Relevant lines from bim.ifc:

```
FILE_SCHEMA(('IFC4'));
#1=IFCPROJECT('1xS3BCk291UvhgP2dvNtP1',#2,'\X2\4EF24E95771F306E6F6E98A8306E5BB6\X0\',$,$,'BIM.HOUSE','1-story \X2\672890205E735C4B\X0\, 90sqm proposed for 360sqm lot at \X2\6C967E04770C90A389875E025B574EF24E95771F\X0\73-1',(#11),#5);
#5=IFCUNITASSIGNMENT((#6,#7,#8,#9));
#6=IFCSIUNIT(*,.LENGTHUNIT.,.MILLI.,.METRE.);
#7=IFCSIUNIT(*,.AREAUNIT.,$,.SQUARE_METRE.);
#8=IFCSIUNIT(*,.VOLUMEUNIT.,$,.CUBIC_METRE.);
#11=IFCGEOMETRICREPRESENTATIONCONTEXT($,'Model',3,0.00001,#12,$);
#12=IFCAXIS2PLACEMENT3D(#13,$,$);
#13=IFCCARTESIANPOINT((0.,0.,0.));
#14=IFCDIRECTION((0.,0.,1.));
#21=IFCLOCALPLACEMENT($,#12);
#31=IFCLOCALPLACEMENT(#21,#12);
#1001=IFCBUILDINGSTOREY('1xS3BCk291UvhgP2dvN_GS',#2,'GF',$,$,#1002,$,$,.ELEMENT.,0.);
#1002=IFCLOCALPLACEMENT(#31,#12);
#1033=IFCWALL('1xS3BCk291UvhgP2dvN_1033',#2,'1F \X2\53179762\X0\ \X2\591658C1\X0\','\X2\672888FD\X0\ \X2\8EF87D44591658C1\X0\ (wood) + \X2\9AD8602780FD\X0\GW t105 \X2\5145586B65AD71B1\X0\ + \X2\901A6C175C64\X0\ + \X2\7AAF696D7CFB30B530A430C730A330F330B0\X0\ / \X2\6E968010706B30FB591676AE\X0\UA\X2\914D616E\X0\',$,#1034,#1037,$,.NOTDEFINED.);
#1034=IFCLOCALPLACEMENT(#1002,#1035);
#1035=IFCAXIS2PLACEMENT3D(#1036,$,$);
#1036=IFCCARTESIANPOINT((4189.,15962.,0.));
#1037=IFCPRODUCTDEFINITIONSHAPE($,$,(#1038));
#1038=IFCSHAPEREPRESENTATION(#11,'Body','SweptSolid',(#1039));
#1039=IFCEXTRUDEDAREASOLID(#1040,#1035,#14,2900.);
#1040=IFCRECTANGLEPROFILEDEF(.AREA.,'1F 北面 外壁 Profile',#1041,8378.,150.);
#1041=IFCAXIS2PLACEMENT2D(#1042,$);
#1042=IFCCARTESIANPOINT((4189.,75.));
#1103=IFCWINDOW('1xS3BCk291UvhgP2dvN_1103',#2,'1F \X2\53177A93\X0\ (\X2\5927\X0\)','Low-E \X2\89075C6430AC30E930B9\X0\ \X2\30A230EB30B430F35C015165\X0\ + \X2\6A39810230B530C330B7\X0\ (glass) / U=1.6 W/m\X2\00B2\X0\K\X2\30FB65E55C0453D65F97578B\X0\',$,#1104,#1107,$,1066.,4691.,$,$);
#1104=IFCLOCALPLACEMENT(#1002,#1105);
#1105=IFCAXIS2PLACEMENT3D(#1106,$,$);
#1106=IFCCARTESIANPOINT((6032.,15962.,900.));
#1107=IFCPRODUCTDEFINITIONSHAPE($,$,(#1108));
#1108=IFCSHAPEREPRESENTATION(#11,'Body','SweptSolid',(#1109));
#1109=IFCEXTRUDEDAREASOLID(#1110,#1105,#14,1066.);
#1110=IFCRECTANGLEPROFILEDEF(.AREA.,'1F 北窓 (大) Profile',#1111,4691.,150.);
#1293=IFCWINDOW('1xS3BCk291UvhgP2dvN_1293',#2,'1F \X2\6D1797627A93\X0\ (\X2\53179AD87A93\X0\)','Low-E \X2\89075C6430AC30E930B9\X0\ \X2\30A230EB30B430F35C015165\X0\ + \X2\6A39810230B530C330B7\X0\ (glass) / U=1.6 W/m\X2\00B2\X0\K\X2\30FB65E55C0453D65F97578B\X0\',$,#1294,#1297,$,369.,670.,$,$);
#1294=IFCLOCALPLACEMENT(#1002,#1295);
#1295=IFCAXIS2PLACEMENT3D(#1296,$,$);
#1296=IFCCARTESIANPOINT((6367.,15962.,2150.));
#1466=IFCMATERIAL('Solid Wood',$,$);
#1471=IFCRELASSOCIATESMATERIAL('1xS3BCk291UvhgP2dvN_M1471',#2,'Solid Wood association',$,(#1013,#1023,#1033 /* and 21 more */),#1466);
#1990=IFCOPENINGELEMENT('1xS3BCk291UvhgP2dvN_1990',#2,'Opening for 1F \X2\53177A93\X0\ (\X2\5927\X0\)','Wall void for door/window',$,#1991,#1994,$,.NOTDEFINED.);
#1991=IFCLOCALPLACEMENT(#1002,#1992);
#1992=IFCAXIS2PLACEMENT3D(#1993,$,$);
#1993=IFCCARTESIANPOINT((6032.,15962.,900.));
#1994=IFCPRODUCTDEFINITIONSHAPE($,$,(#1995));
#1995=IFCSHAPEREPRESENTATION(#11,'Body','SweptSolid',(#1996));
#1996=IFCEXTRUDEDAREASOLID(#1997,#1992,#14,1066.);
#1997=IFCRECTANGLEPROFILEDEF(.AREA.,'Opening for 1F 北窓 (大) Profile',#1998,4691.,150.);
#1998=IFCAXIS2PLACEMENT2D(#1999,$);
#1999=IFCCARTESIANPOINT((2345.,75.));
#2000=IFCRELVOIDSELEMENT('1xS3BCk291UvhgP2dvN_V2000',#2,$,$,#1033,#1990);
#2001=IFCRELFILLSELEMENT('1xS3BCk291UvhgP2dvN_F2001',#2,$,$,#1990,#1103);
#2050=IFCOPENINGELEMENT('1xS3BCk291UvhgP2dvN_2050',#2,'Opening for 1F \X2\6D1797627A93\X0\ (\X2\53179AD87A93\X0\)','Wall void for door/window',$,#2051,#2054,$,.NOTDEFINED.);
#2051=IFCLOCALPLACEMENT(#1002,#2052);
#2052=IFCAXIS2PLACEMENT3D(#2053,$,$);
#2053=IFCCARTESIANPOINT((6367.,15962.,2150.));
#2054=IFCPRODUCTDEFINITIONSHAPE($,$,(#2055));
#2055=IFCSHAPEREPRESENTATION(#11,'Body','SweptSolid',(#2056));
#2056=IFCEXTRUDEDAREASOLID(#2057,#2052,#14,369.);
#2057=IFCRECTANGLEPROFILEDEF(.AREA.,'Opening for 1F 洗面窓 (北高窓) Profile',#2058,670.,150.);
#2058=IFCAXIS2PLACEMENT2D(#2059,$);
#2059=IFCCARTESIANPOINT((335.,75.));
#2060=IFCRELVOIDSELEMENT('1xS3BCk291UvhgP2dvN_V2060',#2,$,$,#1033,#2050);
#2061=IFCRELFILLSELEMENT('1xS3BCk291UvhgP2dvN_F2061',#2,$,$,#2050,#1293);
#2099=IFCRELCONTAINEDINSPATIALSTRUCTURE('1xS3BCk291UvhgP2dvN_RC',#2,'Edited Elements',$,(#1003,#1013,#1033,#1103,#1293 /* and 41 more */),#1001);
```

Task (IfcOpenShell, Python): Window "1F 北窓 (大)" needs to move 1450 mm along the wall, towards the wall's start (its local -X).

```python
import ifcopenshell
import ifcopenshell.api.geometry
import ifcopenshell.util.placement
import ifcopenshell.util.unit

model = ifcopenshell.open("bim.ifc")
unit_scale = ifcopenshell.util.unit.calculate_unit_scale(model)

window = model.by_guid("1xS3BCk291UvhgP2dvN_1103")
opening = window.FillsVoids[0].RelatingOpeningElement
wall = opening.VoidsElements[0].RelatingBuildingElement

wall_matrix = ifcopenshell.util.placement.get_local_placement(wall.ObjectPlacement)
shift = wall_matrix[:3, 0] * -1.45 / unit_scale
before = ifcopenshell.util.placement.get_local_placement(window.ObjectPlacement)[:3, 3].copy()

# The window is not placed relative to its opening, so move both.
for product in (opening, window):
    matrix = ifcopenshell.util.placement.get_local_placement(product.ObjectPlacement)
    matrix[:3, 3] += shift
    ifcopenshell.api.geometry.edit_object_placement(model, product=product, matrix=matrix, is_si=False)

after = ifcopenshell.util.placement.get_local_placement(window.ObjectPlacement)[:3, 3]
print("window moved by", (after - before).round(3) + 0.0)

model.write("bim_updated.ifc")
```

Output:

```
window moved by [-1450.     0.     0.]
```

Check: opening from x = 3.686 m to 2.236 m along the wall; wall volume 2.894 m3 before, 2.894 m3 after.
